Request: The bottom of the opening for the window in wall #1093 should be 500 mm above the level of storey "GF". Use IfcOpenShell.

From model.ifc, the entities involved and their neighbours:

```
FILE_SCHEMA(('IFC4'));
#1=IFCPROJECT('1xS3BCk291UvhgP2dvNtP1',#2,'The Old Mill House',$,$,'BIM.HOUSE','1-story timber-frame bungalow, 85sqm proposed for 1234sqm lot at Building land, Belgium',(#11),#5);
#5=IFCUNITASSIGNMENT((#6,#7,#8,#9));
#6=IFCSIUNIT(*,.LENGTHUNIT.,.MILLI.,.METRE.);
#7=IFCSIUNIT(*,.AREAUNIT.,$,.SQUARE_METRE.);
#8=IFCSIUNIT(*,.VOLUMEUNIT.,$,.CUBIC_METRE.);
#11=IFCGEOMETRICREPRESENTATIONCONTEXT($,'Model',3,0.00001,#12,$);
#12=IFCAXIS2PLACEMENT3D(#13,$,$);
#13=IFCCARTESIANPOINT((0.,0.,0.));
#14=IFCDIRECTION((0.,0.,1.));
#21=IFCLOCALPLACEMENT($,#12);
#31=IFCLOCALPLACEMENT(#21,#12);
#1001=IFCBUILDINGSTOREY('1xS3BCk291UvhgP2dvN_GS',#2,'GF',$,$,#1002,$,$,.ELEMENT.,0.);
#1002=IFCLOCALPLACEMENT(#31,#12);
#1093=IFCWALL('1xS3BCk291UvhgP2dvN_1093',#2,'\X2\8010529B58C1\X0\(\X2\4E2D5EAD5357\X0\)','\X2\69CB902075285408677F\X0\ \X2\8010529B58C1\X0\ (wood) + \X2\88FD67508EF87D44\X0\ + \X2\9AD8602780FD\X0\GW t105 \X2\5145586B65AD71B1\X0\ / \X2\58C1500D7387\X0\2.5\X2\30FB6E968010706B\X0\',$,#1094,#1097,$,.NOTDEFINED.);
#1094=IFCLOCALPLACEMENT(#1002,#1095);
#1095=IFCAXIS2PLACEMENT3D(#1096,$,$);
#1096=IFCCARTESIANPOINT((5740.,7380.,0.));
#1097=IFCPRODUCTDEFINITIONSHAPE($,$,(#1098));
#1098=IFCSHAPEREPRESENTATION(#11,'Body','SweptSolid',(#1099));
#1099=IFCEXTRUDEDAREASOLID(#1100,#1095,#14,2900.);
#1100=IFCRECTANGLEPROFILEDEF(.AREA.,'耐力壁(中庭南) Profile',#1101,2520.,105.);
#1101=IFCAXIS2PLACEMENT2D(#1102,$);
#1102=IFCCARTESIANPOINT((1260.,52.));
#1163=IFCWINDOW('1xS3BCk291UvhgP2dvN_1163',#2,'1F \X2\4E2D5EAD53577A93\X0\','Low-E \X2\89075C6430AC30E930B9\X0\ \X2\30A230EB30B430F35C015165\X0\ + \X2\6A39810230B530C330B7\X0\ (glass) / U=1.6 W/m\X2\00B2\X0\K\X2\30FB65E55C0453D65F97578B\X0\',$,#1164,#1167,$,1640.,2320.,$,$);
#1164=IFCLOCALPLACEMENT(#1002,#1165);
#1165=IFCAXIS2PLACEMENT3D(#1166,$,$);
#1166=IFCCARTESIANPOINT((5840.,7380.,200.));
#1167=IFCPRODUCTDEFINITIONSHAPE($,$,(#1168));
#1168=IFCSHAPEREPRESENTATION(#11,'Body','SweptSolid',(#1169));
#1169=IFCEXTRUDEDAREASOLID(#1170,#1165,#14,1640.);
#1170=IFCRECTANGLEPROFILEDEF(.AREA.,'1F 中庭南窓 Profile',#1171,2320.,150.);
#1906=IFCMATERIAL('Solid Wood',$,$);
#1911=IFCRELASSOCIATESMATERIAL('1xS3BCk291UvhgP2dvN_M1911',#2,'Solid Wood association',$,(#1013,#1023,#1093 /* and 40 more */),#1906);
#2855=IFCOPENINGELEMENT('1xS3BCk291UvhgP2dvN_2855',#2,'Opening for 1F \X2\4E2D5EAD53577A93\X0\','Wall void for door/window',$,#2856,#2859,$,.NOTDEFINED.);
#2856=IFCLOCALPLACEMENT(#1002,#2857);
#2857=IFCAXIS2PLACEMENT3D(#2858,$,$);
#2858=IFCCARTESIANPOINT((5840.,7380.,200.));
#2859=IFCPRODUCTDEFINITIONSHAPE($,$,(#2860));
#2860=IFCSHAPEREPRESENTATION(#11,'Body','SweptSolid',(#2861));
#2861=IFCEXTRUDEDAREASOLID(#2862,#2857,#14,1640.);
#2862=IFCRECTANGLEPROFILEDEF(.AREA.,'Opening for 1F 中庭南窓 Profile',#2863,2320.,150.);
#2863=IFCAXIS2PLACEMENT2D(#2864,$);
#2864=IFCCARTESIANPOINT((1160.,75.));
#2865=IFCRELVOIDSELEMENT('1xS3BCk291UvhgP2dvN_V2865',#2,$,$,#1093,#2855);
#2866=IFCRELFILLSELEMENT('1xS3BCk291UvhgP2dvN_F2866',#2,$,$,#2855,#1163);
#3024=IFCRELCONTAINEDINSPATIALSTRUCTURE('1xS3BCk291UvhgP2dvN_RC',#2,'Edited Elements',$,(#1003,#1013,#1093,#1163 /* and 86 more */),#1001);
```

```python
import numpy as np
import ifcopenshell
import ifcopenshell.api.geometry
import ifcopenshell.geom
import ifcopenshell.util.element
import ifcopenshell.util.placement
import ifcopenshell.util.shape
import ifcopenshell.util.unit

model = ifcopenshell.open("model.ifc")
unit_scale = ifcopenshell.util.unit.calculate_unit_scale(model)

window = model.by_guid("1xS3BCk291UvhgP2dvN_1163")
opening = window.FillsVoids[0].RelatingOpeningElement
storey = ifcopenshell.util.element.get_container(window, ifc_class="IfcBuildingStorey")
level = ifcopenshell.util.placement.get_local_placement(storey.ObjectPlacement)[2, 3]

# The opening's origin need not be at the sill, so measure its lowest point.
shape = ifcopenshell.geom.create_shape(ifcopenshell.geom.settings(), opening)
bottom = ifcopenshell.util.shape.get_shape_bottom_elevation(shape, shape.geometry) / unit_scale
dz = level + 0.5 / unit_scale - bottom

shift = np.array([0.0, 0.0, dz])
# The window is not placed relative to its opening, so move both.
for product in (opening, window):
    matrix = ifcopenshell.util.placement.get_local_placement(product.ObjectPlacement)
    matrix[:3, 3] += shift
    ifcopenshell.api.geometry.edit_object_placement(model, product=product, matrix=matrix, is_si=False)

print(f"moved by {dz * unit_scale:+.3f} m")

model.write("model_v2.ifc")
```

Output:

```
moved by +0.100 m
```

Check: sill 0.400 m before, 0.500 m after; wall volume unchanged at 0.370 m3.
